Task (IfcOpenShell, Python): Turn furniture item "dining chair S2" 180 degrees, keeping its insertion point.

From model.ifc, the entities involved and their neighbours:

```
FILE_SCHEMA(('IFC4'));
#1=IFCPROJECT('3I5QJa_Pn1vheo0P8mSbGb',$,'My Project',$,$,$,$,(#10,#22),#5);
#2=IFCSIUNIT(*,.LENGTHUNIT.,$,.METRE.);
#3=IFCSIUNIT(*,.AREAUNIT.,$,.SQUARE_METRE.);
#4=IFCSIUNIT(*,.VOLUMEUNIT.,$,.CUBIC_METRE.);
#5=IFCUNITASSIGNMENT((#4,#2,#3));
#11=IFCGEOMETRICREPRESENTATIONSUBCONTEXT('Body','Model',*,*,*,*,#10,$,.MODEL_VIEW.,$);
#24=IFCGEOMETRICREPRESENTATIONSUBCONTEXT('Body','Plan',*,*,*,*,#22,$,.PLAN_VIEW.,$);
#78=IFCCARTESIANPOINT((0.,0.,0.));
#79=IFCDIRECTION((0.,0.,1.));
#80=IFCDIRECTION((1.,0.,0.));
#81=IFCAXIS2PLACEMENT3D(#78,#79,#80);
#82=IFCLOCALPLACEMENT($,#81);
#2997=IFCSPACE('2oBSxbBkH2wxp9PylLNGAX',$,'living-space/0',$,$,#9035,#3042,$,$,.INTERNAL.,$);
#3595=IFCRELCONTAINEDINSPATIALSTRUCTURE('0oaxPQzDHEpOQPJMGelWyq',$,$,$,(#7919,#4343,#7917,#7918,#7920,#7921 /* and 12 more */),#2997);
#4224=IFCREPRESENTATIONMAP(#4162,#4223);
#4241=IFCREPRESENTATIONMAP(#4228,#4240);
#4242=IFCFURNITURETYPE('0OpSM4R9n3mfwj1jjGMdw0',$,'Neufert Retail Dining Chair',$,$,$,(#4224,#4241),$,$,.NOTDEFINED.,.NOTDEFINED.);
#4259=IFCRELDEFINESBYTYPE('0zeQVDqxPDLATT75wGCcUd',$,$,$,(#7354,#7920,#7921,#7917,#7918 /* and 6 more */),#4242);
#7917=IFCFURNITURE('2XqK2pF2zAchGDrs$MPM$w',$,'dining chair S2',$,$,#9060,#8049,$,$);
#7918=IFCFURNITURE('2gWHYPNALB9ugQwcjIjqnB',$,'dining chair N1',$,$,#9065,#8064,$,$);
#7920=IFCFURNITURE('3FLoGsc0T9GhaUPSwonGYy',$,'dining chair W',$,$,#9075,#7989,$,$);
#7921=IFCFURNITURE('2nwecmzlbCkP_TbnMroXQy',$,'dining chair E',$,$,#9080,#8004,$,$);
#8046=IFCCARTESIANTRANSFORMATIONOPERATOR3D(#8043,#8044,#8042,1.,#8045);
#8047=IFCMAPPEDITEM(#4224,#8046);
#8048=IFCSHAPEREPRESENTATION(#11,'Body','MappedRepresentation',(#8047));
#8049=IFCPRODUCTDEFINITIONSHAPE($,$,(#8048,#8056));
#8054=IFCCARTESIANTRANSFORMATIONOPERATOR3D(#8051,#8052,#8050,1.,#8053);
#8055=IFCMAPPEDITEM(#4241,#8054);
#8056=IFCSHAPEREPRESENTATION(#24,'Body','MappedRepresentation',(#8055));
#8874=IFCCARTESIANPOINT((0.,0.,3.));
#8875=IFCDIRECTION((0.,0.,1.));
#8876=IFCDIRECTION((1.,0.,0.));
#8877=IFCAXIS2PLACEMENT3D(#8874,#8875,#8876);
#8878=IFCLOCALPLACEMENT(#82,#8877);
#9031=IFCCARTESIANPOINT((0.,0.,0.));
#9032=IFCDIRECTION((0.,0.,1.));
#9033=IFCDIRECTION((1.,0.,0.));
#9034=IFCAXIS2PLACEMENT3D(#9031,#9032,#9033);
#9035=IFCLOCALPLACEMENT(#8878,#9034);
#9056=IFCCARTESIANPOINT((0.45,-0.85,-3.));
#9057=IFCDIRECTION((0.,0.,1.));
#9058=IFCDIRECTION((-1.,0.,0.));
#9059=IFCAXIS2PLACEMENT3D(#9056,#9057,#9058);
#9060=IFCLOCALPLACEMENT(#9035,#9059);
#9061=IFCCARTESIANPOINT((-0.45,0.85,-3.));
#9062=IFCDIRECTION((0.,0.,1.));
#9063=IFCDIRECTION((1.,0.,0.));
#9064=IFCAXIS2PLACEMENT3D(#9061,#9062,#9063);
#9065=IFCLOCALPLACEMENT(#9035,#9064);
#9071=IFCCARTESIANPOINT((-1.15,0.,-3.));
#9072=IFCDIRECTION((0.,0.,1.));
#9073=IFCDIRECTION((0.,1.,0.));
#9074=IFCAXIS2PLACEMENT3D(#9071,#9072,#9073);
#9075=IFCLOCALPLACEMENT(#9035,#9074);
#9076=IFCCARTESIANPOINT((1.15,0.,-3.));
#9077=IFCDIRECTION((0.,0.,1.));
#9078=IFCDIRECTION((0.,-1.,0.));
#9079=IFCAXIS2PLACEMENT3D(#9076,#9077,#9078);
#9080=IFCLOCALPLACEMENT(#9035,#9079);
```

```python
import ifcopenshell
import ifcopenshell.api.geometry
import ifcopenshell.util.placement

model = ifcopenshell.open("model.ifc")

item = model.by_guid("2XqK2pF2zAchGDrs$MPM$w")
matrix = ifcopenshell.util.placement.get_local_placement(item.ObjectPlacement)
matrix = matrix @ ifcopenshell.util.placement.rotation(180, "Z")
ifcopenshell.api.geometry.edit_object_placement(model, product=item, matrix=matrix, is_si=False)

print(ifcopenshell.util.placement.get_local_placement(item.ObjectPlacement).round(3) + 0.0)

model.write("model_updated.ifc")
```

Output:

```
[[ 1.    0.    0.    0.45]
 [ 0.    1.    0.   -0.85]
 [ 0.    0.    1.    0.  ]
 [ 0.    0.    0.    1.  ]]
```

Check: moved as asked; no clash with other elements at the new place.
